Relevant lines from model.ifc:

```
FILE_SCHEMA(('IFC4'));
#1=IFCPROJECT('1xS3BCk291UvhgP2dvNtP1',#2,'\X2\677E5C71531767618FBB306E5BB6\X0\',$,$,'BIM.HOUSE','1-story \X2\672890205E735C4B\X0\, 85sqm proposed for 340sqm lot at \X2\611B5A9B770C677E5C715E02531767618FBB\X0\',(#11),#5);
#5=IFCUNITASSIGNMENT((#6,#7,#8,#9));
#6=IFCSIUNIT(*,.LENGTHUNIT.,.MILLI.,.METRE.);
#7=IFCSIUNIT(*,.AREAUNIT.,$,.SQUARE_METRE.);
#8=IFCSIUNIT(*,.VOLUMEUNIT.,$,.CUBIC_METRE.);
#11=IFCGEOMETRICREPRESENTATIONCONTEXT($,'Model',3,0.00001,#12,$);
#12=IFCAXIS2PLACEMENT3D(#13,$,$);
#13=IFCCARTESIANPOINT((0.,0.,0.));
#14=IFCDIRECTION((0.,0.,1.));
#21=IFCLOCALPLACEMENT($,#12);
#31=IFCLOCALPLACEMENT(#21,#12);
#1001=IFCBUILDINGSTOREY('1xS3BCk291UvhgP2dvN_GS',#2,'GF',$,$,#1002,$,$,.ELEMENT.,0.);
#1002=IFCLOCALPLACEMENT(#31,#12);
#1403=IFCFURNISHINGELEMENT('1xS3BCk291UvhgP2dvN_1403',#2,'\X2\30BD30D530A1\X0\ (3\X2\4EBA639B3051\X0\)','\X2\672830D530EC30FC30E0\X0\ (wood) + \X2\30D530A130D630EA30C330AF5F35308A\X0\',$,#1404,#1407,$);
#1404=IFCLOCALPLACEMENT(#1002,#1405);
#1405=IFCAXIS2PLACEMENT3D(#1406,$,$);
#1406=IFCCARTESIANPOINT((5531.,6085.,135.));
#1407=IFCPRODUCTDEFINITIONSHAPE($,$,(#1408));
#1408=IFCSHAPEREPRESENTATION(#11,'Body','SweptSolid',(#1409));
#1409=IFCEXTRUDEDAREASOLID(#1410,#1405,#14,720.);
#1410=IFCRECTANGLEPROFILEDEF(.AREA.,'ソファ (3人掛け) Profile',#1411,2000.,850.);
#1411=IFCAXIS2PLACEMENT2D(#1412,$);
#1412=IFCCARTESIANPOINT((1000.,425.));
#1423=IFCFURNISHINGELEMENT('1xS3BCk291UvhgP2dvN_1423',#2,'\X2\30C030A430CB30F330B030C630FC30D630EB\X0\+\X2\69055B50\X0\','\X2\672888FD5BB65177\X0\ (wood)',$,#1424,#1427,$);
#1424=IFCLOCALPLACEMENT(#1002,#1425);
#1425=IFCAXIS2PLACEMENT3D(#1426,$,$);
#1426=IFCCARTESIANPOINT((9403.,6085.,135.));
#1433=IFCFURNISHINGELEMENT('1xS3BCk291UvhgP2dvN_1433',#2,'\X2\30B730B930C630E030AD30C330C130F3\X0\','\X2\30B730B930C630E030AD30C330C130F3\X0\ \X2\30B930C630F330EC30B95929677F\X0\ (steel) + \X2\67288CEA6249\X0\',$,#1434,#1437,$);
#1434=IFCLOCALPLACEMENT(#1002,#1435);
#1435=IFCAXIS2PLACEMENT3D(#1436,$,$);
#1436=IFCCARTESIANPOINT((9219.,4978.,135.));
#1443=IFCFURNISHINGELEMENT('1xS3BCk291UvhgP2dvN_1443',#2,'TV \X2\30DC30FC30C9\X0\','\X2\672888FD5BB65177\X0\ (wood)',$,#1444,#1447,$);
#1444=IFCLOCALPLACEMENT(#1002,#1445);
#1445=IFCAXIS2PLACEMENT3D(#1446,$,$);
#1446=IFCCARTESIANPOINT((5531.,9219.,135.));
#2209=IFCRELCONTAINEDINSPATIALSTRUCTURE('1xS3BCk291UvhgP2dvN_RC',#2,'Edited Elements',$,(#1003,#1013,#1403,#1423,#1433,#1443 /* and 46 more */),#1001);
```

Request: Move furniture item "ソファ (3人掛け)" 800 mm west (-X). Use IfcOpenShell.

```python
import ifcopenshell
import ifcopenshell.api.geometry
import ifcopenshell.util.placement

model = ifcopenshell.open("model.ifc")

item = model.by_guid("1xS3BCk291UvhgP2dvN_1403")
matrix = ifcopenshell.util.placement.get_local_placement(item.ObjectPlacement)
matrix[0, 3] -= 800.0
ifcopenshell.api.geometry.edit_object_placement(model, product=item, matrix=matrix, is_si=False)

print(ifcopenshell.util.placement.get_local_placement(item.ObjectPlacement).round(3) + 0.0)

model.write("model_edited.ifc")
```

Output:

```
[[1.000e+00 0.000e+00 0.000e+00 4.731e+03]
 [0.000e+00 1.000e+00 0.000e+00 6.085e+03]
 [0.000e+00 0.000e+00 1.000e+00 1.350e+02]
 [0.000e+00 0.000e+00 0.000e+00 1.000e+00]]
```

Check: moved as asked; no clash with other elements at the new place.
